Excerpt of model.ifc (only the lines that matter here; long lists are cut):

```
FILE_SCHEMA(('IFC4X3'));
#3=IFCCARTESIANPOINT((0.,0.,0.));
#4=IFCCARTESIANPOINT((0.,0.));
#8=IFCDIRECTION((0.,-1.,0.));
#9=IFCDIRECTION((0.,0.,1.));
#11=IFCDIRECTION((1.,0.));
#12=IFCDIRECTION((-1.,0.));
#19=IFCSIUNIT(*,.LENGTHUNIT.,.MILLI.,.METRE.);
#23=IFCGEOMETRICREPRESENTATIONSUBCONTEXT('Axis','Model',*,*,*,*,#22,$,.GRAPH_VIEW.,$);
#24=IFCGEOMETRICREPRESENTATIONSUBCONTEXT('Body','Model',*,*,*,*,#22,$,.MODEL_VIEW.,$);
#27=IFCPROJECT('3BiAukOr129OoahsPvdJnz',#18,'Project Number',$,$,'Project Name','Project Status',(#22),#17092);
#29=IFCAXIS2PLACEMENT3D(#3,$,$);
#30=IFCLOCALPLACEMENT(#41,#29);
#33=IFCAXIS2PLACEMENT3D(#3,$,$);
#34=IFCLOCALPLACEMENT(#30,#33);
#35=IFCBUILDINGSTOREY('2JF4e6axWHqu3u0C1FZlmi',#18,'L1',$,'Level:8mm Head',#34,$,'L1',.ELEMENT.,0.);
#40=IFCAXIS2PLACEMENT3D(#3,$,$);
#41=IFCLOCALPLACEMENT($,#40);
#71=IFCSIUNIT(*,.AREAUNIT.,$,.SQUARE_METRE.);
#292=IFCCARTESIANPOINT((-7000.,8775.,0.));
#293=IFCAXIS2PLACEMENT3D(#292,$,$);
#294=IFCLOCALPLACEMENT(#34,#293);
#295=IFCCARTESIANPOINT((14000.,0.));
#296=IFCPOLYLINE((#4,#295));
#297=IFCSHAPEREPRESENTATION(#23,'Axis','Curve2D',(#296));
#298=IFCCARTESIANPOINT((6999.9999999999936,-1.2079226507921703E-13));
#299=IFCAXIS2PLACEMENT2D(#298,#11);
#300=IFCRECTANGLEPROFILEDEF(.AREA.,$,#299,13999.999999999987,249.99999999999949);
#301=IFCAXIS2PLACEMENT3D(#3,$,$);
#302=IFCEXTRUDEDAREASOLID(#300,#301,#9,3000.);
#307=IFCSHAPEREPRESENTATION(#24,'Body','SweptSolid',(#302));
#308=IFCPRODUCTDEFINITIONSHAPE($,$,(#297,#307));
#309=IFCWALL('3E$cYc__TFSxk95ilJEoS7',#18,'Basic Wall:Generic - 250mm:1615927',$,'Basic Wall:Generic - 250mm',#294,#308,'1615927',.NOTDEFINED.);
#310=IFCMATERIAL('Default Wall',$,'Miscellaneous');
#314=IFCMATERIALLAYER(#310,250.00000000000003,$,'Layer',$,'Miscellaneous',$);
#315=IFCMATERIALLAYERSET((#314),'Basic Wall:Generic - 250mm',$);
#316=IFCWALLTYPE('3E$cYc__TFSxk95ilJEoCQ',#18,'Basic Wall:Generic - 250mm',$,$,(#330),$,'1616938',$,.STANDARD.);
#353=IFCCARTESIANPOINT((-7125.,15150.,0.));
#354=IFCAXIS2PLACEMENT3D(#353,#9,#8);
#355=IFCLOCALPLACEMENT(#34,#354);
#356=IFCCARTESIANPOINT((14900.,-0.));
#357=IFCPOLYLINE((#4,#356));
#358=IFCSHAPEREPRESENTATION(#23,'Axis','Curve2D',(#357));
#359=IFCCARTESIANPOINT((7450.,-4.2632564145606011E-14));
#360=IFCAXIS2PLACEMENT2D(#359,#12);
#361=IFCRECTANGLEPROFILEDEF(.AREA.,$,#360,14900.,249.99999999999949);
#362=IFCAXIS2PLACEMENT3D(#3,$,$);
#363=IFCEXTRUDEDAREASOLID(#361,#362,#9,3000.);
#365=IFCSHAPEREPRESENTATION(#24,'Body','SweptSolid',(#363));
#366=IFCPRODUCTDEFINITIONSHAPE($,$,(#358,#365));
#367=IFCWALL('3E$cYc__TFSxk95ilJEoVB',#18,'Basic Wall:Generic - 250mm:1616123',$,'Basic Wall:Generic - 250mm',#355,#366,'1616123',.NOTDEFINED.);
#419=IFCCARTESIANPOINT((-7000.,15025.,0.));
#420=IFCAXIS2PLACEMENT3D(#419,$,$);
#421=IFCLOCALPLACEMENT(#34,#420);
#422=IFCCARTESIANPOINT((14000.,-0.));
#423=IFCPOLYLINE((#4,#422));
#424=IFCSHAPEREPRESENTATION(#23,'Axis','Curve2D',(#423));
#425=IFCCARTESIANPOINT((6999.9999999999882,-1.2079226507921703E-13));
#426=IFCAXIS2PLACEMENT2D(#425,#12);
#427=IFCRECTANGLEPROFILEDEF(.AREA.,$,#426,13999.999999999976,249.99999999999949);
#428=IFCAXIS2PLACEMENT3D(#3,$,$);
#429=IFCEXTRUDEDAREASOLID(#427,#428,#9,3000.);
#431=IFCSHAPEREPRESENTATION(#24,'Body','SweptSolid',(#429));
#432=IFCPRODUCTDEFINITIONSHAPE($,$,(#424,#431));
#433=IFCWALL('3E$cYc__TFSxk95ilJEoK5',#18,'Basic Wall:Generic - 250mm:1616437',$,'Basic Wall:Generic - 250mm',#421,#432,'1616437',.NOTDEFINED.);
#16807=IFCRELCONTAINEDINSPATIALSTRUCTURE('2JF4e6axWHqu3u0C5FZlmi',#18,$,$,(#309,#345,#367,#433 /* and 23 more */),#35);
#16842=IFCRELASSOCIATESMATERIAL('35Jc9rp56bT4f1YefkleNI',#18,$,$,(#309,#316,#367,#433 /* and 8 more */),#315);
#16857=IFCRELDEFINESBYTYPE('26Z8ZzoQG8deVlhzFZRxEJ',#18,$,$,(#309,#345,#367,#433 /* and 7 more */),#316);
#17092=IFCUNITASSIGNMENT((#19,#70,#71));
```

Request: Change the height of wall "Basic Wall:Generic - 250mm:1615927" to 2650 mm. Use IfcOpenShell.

```python
import ifcopenshell
import ifcopenshell.geom
import ifcopenshell.util.representation
import ifcopenshell.util.shape

model = ifcopenshell.open("model.ifc")
settings = ifcopenshell.geom.settings()


def volume(element):
    """Net volume in cubic metres, openings subtracted."""
    shape = ifcopenshell.geom.create_shape(settings, element)
    return ifcopenshell.util.shape.get_volume(shape.geometry)


wall = model.by_id(309)
before = volume(wall)

body = ifcopenshell.util.representation.get_representation(wall, "Model", "Body")
solid = body.Items[0]
old_height = solid.Depth
solid.Depth = 2650.0
after = volume(wall)

print(f"height {old_height:g} -> {solid.Depth:g}, volume {before:.3f} -> {after:.3f} m3")

model.write("model_updated.ifc")
```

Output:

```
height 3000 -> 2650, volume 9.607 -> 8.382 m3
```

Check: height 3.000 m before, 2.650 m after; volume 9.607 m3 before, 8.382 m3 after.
